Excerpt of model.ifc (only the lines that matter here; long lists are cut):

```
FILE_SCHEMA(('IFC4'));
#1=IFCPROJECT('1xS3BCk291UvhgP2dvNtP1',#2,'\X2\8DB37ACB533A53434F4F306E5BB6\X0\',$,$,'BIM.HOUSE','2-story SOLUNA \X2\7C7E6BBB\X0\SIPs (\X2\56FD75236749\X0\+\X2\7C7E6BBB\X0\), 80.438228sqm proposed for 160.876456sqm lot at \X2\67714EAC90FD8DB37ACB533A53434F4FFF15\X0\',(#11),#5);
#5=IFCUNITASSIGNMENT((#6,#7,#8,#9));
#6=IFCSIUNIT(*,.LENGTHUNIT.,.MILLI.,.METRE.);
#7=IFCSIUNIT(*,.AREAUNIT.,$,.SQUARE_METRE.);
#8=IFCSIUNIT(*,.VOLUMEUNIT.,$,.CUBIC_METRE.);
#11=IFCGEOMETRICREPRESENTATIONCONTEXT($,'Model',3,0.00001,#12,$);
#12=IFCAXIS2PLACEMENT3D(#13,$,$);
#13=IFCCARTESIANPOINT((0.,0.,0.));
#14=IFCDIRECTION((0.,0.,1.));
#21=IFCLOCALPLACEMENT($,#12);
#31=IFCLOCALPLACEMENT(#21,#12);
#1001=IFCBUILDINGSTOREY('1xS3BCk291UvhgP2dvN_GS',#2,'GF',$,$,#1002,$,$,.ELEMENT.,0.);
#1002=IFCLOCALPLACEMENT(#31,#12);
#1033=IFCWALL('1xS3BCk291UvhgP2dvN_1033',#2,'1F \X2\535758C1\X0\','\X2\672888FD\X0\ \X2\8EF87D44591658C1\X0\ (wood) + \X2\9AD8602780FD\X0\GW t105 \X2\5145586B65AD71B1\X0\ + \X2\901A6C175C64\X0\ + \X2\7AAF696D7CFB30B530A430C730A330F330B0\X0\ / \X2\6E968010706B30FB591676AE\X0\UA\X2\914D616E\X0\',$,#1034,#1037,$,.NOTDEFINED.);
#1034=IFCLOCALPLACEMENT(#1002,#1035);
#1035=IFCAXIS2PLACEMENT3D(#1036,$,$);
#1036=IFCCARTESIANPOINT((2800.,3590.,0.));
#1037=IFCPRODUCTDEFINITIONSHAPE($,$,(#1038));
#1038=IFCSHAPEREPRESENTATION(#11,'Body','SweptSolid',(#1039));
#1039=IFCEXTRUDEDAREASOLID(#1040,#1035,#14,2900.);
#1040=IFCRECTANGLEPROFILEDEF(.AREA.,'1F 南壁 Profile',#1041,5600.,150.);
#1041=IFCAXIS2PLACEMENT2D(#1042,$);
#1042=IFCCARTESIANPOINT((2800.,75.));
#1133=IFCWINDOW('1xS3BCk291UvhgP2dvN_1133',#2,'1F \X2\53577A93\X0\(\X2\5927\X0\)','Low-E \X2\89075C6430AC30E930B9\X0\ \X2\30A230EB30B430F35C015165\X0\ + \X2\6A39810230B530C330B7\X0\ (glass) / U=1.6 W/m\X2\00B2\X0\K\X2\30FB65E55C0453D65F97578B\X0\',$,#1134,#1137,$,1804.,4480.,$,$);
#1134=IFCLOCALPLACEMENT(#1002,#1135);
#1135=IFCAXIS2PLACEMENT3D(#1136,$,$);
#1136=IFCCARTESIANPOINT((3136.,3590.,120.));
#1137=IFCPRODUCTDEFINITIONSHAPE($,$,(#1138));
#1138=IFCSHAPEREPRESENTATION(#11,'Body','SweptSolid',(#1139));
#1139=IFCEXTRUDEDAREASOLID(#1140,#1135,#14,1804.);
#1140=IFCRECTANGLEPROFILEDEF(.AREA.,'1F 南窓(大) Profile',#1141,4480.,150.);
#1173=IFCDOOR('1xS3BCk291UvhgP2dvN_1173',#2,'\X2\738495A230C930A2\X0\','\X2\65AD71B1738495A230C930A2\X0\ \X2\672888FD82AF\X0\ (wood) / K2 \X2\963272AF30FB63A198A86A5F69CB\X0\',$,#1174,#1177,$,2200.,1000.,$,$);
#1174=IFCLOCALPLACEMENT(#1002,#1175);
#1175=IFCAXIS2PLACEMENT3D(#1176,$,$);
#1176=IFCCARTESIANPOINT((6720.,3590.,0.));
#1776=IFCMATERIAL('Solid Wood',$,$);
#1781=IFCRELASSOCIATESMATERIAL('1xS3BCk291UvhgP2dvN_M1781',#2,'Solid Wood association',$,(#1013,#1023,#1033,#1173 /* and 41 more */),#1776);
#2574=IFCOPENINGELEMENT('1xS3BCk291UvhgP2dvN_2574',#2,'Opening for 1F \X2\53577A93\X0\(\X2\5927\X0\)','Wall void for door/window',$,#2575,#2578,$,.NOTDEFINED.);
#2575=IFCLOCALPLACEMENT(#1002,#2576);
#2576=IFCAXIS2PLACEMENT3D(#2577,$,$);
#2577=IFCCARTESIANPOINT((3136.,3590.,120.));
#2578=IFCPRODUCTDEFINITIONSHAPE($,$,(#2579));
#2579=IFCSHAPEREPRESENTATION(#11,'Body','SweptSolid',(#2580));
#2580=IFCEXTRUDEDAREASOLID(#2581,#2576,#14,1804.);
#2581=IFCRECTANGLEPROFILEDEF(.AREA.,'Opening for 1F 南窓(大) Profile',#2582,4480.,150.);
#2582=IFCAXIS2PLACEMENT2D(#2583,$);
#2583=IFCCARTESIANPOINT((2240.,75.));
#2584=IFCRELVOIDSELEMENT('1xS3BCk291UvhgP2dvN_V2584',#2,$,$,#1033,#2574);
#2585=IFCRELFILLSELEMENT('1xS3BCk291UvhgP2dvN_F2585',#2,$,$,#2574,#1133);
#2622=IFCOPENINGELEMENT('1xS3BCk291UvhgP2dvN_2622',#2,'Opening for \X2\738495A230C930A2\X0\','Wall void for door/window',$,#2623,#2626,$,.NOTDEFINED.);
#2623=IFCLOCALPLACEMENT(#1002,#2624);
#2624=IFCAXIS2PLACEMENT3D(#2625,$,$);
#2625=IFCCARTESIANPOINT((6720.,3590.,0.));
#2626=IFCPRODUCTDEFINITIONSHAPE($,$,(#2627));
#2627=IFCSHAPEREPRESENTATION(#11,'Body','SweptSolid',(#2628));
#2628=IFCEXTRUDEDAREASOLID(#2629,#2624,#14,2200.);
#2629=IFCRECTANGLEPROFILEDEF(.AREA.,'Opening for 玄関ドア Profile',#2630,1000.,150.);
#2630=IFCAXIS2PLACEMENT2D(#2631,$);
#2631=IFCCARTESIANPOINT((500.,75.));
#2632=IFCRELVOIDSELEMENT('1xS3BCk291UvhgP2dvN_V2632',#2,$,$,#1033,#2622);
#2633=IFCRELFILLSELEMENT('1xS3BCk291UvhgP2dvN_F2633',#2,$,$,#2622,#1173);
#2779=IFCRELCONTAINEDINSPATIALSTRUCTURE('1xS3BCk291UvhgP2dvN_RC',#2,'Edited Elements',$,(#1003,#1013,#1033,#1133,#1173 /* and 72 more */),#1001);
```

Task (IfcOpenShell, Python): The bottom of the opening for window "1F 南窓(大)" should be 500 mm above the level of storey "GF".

```python
import numpy as np
import ifcopenshell
import ifcopenshell.api.geometry
import ifcopenshell.geom
import ifcopenshell.util.element
import ifcopenshell.util.placement
import ifcopenshell.util.shape
import ifcopenshell.util.unit

model = ifcopenshell.open("model.ifc")
unit_scale = ifcopenshell.util.unit.calculate_unit_scale(model)

window = model.by_guid("1xS3BCk291UvhgP2dvN_1133")
opening = window.FillsVoids[0].RelatingOpeningElement
storey = ifcopenshell.util.element.get_container(window, ifc_class="IfcBuildingStorey")
level = ifcopenshell.util.placement.get_local_placement(storey.ObjectPlacement)[2, 3]

# The opening's origin need not be at the sill, so measure its lowest point.
shape = ifcopenshell.geom.create_shape(ifcopenshell.geom.settings(), opening)
bottom = ifcopenshell.util.shape.get_shape_bottom_elevation(shape, shape.geometry) / unit_scale
dz = level + 500.0 - bottom

shift = np.array([0.0, 0.0, dz])
# The window is not placed relative to its opening, so move both.
for product in (opening, window):
    matrix = ifcopenshell.util.placement.get_local_placement(product.ObjectPlacement)
    matrix[:3, 3] += shift
    ifcopenshell.api.geometry.edit_object_placement(model, product=product, matrix=matrix, is_si=False)

print(f"moved by {dz * unit_scale:+.3f} m")

model.write("model_edited.ifc")
```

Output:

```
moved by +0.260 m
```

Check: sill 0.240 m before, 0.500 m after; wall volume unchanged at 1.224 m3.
